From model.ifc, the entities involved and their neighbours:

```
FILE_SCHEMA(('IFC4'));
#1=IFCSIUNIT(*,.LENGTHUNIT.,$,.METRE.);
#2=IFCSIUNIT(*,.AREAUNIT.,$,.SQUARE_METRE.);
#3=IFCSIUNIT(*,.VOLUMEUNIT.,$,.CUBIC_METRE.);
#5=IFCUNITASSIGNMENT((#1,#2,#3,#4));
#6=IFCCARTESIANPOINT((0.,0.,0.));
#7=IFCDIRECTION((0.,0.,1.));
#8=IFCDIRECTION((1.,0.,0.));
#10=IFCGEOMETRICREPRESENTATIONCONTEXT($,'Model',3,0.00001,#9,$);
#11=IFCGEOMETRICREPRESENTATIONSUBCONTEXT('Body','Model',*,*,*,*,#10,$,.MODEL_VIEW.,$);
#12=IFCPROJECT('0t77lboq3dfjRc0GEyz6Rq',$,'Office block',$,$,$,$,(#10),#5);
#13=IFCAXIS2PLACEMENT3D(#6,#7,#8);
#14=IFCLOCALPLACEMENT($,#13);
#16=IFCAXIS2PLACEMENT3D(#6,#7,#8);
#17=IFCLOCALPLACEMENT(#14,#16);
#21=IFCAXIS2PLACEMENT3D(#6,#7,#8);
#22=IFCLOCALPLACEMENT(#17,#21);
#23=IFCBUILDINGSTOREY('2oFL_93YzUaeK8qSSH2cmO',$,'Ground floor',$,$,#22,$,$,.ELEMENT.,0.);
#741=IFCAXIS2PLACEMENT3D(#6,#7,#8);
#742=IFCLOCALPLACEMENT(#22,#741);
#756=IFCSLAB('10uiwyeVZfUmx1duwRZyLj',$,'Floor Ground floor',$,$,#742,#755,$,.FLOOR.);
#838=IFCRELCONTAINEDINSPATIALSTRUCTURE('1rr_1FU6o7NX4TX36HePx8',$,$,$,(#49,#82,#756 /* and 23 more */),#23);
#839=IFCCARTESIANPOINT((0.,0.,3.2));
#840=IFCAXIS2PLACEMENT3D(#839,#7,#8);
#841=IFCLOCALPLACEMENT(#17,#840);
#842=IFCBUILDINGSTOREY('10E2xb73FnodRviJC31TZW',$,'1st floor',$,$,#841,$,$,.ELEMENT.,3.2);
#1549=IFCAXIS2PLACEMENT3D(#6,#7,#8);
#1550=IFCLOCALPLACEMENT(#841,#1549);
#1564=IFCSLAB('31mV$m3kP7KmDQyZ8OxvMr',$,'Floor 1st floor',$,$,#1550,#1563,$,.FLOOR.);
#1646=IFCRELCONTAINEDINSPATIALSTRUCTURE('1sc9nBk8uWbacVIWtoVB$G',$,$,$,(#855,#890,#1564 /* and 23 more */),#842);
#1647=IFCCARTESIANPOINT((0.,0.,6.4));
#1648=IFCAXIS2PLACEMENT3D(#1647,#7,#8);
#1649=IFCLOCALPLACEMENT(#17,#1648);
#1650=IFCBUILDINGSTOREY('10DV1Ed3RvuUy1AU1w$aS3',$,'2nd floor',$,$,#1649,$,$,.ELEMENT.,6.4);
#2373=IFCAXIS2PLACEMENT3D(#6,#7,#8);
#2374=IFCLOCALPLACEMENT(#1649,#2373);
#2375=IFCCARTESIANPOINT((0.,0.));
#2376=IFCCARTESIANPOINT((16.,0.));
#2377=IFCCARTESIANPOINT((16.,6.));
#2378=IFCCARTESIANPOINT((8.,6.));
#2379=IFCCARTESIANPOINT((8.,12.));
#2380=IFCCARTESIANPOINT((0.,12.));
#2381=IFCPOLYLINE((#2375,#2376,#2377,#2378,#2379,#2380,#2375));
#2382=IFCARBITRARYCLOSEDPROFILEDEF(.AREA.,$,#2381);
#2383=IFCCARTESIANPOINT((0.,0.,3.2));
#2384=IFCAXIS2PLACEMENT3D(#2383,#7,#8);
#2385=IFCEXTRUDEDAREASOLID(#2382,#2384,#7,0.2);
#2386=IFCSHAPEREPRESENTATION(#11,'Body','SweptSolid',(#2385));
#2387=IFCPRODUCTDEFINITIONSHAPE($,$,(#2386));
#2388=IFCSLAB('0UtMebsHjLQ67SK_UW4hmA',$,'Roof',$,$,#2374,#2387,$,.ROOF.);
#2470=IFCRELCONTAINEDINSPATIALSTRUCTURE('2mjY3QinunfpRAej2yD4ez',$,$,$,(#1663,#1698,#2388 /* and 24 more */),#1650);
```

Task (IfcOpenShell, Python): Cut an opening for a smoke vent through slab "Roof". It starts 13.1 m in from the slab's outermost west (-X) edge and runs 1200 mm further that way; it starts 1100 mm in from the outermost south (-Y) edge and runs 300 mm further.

```python
import numpy as np
import ifcopenshell
import ifcopenshell.api.feature
import ifcopenshell.api.geometry
import ifcopenshell.api.root
import ifcopenshell.geom
import ifcopenshell.util.placement
import ifcopenshell.util.representation
import ifcopenshell.util.shape
import ifcopenshell.util.unit

model = ifcopenshell.open("model.ifc")
unit_scale = ifcopenshell.util.unit.calculate_unit_scale(model)
settings = ifcopenshell.geom.settings()


def volume(element):
    """Net volume in cubic metres, openings subtracted."""
    shape = ifcopenshell.geom.create_shape(settings, element)
    return ifcopenshell.util.shape.get_volume(shape.geometry)


slab = model.by_guid("0UtMebsHjLQ67SK_UW4hmA")
before = volume(slab)

# Extent in the slab's own axes, in metres. The edges named are its -X and -Y sides.
slab_shape = ifcopenshell.geom.create_shape(settings, slab)
vertices = ifcopenshell.util.shape.get_vertices(slab_shape.geometry)
x_min, y_min, bottom = vertices.min(axis=0)
top = vertices[:, 2].max()

opening = ifcopenshell.api.root.create_entity(model, ifc_class="IfcOpeningElement", name="Smoke vent opening", predefined_type="OPENING")
context = ifcopenshell.util.representation.get_context(model, "Model", "Body", "MODEL_VIEW")
width, depth = 1.2, 0.3
outline = [(0.0, 0.0), (width, 0.0), (width, depth), (0.0, depth), (0.0, 0.0)]
# Overshoot both faces by 50 mm so the cut is clean.
shape = ifcopenshell.api.geometry.add_slab_representation(
    model, context=context, depth=top - bottom + 0.1, polyline=outline
)
ifcopenshell.api.geometry.assign_representation(model, product=opening, representation=shape)

matrix = ifcopenshell.util.placement.get_local_placement(slab.ObjectPlacement)
matrix[:, 3] = matrix @ np.append(np.array([x_min + 13.1, y_min + 1.1, bottom - 0.05]) / unit_scale, 1.0)
ifcopenshell.api.geometry.edit_object_placement(model, product=opening, matrix=matrix, is_si=False)
ifcopenshell.api.feature.add_feature(model, feature=opening, element=slab)

after = volume(slab)

print(f"slab volume {before:.3f} -> {after:.3f} m3")

model.write("model-out.ifc")
```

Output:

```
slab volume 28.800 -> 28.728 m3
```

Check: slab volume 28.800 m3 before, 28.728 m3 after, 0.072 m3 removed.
